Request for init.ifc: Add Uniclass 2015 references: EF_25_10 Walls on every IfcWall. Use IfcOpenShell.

First a look at what the model holds.

```python
import ifcopenshell

model = ifcopenshell.open("init.ifc")
print(model.schema)
print("classifications:", [c.Name for c in model.by_type("IfcClassification")])
for ifc_class in ("IfcDoor", "IfcRoof", "IfcStair", "IfcWall", "IfcWindow"):
    print(ifc_class, len(model.by_type(ifc_class)))
```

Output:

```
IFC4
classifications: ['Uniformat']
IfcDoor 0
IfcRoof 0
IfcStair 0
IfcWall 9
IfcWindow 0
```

```python
import ifcopenshell
import ifcopenshell.api.classification

model = ifcopenshell.open("init.ifc")

system = ifcopenshell.api.classification.add_classification(model, classification="Uniclass 2015")

codes = {
    "IfcWall": ("EF_25_10", "Walls"),
}
for ifc_class, (code, name) in codes.items():
    products = model.by_type(ifc_class)
    ifcopenshell.api.classification.add_reference(
        model, products=products, classification=system, identification=code, name=name
    )
    print(code, len(products))

model.write("init_v2.ifc")
```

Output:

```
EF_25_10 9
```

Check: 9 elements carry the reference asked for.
